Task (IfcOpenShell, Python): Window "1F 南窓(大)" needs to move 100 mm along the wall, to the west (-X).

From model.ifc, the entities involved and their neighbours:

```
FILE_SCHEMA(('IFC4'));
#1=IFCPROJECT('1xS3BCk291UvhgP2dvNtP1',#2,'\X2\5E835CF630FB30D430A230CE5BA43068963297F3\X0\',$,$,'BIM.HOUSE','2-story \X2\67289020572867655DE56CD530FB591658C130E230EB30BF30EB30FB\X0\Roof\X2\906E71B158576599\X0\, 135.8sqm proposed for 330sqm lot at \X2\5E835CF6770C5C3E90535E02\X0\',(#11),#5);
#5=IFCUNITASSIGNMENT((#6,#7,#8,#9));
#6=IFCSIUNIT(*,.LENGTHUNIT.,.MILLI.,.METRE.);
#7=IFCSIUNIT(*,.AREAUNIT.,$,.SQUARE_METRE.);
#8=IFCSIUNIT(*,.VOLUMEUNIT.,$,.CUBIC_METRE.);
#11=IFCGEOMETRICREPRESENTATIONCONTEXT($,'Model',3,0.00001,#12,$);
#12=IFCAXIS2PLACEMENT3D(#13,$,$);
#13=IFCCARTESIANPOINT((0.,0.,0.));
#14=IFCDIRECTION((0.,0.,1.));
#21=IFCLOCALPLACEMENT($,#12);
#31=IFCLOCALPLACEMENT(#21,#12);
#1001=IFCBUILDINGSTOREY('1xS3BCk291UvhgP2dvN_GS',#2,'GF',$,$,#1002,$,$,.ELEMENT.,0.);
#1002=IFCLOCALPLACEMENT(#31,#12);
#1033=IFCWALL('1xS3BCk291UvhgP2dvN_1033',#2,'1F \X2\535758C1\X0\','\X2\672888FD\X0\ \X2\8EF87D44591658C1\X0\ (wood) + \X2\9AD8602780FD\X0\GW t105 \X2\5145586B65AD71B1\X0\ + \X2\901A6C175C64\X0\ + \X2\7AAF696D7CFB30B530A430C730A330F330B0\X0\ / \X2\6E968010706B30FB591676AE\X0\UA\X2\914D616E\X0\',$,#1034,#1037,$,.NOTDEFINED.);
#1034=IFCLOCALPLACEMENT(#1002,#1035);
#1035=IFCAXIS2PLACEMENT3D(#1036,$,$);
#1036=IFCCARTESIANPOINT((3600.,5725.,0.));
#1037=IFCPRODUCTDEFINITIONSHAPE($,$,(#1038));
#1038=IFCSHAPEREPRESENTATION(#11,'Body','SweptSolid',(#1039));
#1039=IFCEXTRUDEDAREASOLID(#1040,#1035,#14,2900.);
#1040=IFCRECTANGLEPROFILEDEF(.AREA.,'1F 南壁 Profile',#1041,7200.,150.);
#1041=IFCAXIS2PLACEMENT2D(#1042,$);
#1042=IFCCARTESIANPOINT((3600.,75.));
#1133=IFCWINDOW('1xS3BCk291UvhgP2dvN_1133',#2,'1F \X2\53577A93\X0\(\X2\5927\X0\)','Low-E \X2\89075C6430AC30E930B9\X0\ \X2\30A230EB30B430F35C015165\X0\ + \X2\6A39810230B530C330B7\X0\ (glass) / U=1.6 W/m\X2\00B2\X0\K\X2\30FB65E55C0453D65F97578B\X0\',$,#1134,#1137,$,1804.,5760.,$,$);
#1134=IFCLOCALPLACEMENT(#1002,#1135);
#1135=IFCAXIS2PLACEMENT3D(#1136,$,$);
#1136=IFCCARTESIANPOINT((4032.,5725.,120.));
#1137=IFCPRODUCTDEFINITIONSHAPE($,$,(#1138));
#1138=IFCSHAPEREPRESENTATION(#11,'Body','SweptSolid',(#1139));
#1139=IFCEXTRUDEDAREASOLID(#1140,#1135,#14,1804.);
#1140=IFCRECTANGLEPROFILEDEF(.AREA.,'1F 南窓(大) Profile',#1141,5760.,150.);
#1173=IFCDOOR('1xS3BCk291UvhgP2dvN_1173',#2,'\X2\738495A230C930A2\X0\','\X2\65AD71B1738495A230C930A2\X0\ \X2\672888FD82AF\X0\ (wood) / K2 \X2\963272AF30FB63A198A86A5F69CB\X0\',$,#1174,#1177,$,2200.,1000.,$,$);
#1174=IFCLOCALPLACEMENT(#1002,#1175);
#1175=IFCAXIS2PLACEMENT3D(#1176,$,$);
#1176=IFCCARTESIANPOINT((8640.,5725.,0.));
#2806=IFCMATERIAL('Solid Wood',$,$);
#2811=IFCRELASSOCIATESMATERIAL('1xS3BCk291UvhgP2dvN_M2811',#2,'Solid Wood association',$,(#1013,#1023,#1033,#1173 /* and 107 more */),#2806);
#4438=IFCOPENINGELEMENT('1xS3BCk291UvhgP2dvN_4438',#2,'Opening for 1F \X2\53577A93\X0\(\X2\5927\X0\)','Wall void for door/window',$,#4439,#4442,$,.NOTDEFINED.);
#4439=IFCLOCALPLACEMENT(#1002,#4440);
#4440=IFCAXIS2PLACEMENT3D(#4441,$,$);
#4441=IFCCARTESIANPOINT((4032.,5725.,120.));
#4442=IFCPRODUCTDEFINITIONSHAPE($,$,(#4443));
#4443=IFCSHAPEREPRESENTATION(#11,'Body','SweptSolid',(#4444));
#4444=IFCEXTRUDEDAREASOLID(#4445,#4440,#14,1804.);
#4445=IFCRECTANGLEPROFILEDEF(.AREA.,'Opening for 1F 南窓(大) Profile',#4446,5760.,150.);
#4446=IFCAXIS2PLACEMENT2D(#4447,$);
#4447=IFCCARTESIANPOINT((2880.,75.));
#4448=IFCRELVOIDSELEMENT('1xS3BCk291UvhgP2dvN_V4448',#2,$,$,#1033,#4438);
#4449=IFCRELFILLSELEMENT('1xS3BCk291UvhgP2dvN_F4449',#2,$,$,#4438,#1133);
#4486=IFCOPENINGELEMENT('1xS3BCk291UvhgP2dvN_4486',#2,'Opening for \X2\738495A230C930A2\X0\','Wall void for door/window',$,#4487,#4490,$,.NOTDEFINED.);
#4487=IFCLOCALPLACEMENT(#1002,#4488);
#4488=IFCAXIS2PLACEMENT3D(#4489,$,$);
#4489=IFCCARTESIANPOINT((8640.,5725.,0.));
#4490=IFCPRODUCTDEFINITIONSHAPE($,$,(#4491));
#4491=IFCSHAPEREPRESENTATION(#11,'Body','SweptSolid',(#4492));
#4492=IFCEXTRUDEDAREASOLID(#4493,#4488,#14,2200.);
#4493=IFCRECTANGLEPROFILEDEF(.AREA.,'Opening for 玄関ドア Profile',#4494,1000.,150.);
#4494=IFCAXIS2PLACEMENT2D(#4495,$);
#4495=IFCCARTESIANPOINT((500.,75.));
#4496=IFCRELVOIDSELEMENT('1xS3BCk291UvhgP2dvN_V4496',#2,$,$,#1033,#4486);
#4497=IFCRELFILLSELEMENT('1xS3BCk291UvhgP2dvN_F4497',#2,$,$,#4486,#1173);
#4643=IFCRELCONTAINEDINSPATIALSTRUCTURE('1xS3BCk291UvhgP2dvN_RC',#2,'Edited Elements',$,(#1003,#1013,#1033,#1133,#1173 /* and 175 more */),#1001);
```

```python
import ifcopenshell
import ifcopenshell.api.geometry
import ifcopenshell.util.placement
import ifcopenshell.util.unit

model = ifcopenshell.open("model.ifc")
unit_scale = ifcopenshell.util.unit.calculate_unit_scale(model)

window = model.by_id(1133)
opening = window.FillsVoids[0].RelatingOpeningElement
wall = opening.VoidsElements[0].RelatingBuildingElement

wall_matrix = ifcopenshell.util.placement.get_local_placement(wall.ObjectPlacement)
shift = wall_matrix[:3, 0] * -0.1 / unit_scale
before = ifcopenshell.util.placement.get_local_placement(window.ObjectPlacement)[:3, 3].copy()

# The window is not placed relative to its opening, so move both.
for product in (opening, window):
    matrix = ifcopenshell.util.placement.get_local_placement(product.ObjectPlacement)
    matrix[:3, 3] += shift
    ifcopenshell.api.geometry.edit_object_placement(model, product=product, matrix=matrix, is_si=False)

after = ifcopenshell.util.placement.get_local_placement(window.ObjectPlacement)[:3, 3]
print("window moved by", (after - before).round(3) + 0.0)

model.write("model-out.ifc")
```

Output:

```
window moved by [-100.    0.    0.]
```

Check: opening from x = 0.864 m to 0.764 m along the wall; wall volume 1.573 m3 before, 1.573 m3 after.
